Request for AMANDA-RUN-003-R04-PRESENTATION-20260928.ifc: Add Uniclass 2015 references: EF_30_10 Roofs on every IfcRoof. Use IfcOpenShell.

First a look at what the model holds.

```python
import ifcopenshell

model = ifcopenshell.open("AMANDA-RUN-003-R04-PRESENTATION-20260928.ifc")
print(model.schema)
print("classifications:", [c.Name for c in model.by_type("IfcClassification")])
for ifc_class in ("IfcDoor", "IfcRoof", "IfcStair", "IfcWall", "IfcWindow"):
    print(ifc_class, len(model.by_type(ifc_class)))
```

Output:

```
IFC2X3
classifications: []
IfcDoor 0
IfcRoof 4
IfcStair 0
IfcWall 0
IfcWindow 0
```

```python
import ifcopenshell
import ifcopenshell.api.classification

model = ifcopenshell.open("AMANDA-RUN-003-R04-PRESENTATION-20260928.ifc")

# IFC2X3 requires Source and Edition and has no link from the project to the system.
system = model.create_entity("IfcClassification", Source="NBS", Edition="2015", Name="Uniclass 2015")

codes = {
    "IfcRoof": ("EF_30_10", "Roofs"),
}
for ifc_class, (code, name) in codes.items():
    products = model.by_type(ifc_class)
    ifcopenshell.api.classification.add_reference(
        model, products=products, classification=system, identification=code, name=name
    )
    print(code, len(products))

model.write("AMANDA-RUN-003-R04-PRESENTATION-20260928_v2.ifc")
```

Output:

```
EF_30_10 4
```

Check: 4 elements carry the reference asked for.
